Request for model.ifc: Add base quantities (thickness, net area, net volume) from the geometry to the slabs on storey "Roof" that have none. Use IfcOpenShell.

First a look at what the model holds.

```python
import ifcopenshell
import ifcopenshell.util.element
import ifcopenshell.util.unit

model = ifcopenshell.open("model.ifc")
print(model.schema)
for unit_type in ("LENGTHUNIT", "AREAUNIT", "VOLUMEUNIT"):
    print(unit_type, ifcopenshell.util.unit.calculate_unit_scale(model, unit_type))
storey = next(s for s in model.by_type("IfcBuildingStorey") if s.Name == "Roof")
slabs = [e for e in ifcopenshell.util.element.get_decomposition(storey) if e.is_a("IfcSlab")]
for e in sorted(slabs, key=lambda e: e.id()):
    print(e.id(), e.is_a(), e.Name, list(ifcopenshell.util.element.get_psets(e, qtos_only=True)), sep=" | ")
```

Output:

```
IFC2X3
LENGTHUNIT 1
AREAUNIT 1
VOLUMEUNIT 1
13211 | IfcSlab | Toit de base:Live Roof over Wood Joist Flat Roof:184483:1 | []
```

```python
import ifcopenshell
import ifcopenshell.api.pset
import ifcopenshell.geom
import ifcopenshell.util.element
import ifcopenshell.util.shape
import ifcopenshell.util.unit

model = ifcopenshell.open("model.ifc")
unit_scale = ifcopenshell.util.unit.calculate_unit_scale(model)
area_scale = ifcopenshell.util.unit.calculate_unit_scale(model, "AREAUNIT")
volume_scale = ifcopenshell.util.unit.calculate_unit_scale(model, "VOLUMEUNIT")
settings = ifcopenshell.geom.settings()

storey = next(s for s in model.by_type("IfcBuildingStorey") if s.Name == "Roof")
slabs = [e for e in ifcopenshell.util.element.get_decomposition(storey) if e.is_a("IfcSlab")]

for e in sorted(slabs, key=lambda e: e.id()):
    if ifcopenshell.util.element.get_psets(e, qtos_only=True, should_inherit=False):
        continue
    # Geometry comes back in metres, in the element's own axes.
    shape = ifcopenshell.geom.create_shape(settings, e)
    values = {
        "Width": ifcopenshell.util.shape.get_z(shape.geometry) / unit_scale,
        "NetArea": ifcopenshell.util.shape.get_footprint_area(shape.geometry) / area_scale,
        "NetVolume": ifcopenshell.util.shape.get_volume(shape.geometry) / volume_scale,
    }
    qto = ifcopenshell.api.pset.add_qto(model, product=e, name="BaseQuantities")
    ifcopenshell.api.pset.edit_qto(model, qto=qto, properties=values)
    print(e.id(), {k: round(v, 3) for k, v in values.items()})

model.write("model_rev.ifc")
```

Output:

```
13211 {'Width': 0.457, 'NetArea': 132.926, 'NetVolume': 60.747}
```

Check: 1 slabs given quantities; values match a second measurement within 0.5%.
